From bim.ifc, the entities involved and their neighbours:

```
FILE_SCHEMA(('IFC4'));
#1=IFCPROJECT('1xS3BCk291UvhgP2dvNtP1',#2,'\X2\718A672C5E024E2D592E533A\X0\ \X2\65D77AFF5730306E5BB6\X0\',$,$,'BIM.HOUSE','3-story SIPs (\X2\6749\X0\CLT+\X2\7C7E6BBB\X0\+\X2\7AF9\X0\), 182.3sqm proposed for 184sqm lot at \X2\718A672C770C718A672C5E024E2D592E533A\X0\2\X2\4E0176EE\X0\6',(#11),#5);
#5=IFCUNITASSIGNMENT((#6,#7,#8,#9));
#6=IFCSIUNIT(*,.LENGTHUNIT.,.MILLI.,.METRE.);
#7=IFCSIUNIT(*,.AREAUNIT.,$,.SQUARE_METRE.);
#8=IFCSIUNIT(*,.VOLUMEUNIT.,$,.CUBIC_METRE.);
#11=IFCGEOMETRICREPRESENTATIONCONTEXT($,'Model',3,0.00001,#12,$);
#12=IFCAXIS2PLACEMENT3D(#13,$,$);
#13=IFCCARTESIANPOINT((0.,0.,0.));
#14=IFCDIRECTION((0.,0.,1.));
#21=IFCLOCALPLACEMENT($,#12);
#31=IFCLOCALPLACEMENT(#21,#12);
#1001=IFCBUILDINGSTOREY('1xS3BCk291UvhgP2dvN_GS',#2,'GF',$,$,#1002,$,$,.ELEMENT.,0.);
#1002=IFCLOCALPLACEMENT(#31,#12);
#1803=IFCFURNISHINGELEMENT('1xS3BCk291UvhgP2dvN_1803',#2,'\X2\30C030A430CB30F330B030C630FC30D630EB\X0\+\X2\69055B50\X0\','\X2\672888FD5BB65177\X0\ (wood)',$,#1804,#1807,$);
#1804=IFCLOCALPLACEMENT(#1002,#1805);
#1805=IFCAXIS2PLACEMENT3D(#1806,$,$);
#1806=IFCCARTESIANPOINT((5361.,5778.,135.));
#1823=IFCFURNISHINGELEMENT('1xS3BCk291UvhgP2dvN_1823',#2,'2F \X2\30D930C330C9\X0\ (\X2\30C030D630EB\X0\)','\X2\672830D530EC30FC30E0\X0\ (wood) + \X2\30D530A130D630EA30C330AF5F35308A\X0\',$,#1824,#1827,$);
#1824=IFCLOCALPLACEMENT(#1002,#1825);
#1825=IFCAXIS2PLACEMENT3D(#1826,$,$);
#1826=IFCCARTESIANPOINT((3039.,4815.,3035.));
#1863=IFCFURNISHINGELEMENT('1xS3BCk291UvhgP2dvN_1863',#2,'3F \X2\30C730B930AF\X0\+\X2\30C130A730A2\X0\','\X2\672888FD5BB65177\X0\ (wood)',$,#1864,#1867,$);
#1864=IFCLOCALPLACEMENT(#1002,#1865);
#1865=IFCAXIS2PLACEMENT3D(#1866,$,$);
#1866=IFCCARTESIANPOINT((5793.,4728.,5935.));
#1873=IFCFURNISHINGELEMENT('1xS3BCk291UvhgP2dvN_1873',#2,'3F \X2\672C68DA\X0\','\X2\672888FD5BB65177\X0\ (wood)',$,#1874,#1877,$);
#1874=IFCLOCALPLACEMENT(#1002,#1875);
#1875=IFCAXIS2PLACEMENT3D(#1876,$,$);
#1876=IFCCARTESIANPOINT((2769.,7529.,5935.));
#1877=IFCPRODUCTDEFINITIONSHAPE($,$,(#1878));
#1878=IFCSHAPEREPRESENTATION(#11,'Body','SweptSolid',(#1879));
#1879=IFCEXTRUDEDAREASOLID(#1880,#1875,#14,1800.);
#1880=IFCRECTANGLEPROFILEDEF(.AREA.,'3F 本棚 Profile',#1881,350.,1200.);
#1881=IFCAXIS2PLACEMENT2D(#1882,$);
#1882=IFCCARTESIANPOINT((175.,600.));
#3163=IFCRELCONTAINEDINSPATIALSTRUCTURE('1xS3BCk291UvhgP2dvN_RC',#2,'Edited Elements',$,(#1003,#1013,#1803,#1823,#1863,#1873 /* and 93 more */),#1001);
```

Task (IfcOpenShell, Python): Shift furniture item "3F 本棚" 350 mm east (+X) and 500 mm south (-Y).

```python
import ifcopenshell
import ifcopenshell.api.geometry
import ifcopenshell.util.placement
import ifcopenshell.util.unit

model = ifcopenshell.open("bim.ifc")
unit_scale = ifcopenshell.util.unit.calculate_unit_scale(model)

item = model.by_guid("1xS3BCk291UvhgP2dvN_1873")
matrix = ifcopenshell.util.placement.get_local_placement(item.ObjectPlacement)
matrix[0, 3] += 0.35 / unit_scale
matrix[1, 3] -= 0.5 / unit_scale
ifcopenshell.api.geometry.edit_object_placement(model, product=item, matrix=matrix, is_si=False)

print(ifcopenshell.util.placement.get_local_placement(item.ObjectPlacement).round(3) + 0.0)

model.write("bim_rev.ifc")
```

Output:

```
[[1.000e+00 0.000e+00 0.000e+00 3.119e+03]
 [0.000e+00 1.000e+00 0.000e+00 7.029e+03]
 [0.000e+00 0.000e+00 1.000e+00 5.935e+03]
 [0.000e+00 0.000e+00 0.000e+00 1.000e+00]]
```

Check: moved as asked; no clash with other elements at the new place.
